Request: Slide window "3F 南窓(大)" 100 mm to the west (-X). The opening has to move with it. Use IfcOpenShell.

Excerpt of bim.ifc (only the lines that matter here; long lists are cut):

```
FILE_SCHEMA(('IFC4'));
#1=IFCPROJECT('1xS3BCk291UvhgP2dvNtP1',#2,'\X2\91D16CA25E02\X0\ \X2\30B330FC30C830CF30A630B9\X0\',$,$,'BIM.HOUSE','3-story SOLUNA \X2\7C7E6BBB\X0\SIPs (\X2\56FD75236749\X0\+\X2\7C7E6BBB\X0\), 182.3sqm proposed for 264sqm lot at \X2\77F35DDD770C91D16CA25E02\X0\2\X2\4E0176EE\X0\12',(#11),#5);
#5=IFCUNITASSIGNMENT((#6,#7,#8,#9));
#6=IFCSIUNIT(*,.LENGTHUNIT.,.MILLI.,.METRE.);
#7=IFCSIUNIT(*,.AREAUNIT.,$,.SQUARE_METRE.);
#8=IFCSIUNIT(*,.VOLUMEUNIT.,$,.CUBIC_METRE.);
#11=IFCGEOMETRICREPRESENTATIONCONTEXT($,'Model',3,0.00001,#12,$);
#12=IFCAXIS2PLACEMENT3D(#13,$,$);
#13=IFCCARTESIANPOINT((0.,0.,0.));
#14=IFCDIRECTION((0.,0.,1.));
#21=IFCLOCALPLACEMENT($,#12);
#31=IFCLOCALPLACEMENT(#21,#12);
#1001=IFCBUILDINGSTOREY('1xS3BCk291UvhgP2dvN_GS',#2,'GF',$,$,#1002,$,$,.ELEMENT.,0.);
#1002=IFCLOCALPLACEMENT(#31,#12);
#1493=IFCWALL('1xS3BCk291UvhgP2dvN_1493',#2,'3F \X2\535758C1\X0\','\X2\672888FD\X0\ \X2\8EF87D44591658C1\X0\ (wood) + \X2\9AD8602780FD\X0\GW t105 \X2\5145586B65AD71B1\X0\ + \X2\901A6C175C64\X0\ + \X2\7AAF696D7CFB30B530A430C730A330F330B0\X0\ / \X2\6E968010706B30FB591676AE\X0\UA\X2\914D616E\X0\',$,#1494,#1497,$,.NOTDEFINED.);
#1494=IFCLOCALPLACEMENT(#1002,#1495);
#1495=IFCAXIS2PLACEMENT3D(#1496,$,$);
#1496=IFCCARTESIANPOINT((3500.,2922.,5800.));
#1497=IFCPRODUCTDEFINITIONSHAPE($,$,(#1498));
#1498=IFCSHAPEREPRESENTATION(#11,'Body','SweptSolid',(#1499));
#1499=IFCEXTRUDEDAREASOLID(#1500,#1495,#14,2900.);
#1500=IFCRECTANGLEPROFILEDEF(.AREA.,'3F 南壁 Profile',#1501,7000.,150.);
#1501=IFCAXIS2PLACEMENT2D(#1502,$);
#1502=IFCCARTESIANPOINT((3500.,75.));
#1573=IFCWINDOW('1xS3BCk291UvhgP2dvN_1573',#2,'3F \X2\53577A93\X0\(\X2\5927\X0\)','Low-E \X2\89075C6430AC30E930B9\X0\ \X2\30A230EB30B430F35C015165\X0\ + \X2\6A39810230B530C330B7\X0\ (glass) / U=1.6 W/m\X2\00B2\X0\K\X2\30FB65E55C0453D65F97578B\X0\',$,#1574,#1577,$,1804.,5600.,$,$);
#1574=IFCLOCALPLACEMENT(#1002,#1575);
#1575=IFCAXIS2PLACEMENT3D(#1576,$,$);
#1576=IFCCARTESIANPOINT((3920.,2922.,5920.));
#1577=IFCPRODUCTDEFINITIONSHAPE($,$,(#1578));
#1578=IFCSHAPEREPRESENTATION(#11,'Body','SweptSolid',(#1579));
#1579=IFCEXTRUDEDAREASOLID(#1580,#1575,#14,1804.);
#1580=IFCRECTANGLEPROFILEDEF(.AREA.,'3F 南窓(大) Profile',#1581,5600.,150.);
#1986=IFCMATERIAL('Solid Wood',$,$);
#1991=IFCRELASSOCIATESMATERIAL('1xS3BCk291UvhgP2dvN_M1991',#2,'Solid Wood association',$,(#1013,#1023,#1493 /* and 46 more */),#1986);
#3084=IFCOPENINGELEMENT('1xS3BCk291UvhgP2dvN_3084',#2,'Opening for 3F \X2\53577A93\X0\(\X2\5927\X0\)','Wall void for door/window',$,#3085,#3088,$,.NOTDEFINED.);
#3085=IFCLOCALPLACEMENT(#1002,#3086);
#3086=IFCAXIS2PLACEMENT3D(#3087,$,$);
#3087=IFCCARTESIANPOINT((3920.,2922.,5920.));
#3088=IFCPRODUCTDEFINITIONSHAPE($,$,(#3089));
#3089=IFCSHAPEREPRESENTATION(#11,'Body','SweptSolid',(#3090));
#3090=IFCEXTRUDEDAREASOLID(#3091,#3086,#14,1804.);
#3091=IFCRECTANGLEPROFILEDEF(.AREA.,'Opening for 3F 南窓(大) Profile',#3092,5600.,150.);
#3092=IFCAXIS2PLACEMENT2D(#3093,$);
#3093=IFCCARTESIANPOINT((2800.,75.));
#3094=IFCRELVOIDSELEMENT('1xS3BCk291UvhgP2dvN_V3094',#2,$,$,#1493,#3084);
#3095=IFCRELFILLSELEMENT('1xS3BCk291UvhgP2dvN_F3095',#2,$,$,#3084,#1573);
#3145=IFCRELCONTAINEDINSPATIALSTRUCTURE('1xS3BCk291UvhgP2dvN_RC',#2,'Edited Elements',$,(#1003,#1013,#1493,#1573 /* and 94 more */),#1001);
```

```python
import ifcopenshell
import ifcopenshell.api.geometry
import ifcopenshell.util.placement

model = ifcopenshell.open("bim.ifc")

window = model.by_id(1573)
opening = window.FillsVoids[0].RelatingOpeningElement
wall = opening.VoidsElements[0].RelatingBuildingElement

wall_matrix = ifcopenshell.util.placement.get_local_placement(wall.ObjectPlacement)
shift = wall_matrix[:3, 0] * -100.0
before = ifcopenshell.util.placement.get_local_placement(window.ObjectPlacement)[:3, 3].copy()

# The window is not placed relative to its opening, so move both.
for product in (opening, window):
    matrix = ifcopenshell.util.placement.get_local_placement(product.ObjectPlacement)
    matrix[:3, 3] += shift
    ifcopenshell.api.geometry.edit_object_placement(model, product=product, matrix=matrix, is_si=False)

after = ifcopenshell.util.placement.get_local_placement(window.ObjectPlacement)[:3, 3]
print("window moved by", (after - before).round(3) + 0.0)

model.write("bim-out.ifc")
```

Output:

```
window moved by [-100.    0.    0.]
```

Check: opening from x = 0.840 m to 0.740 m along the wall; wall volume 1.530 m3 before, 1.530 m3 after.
